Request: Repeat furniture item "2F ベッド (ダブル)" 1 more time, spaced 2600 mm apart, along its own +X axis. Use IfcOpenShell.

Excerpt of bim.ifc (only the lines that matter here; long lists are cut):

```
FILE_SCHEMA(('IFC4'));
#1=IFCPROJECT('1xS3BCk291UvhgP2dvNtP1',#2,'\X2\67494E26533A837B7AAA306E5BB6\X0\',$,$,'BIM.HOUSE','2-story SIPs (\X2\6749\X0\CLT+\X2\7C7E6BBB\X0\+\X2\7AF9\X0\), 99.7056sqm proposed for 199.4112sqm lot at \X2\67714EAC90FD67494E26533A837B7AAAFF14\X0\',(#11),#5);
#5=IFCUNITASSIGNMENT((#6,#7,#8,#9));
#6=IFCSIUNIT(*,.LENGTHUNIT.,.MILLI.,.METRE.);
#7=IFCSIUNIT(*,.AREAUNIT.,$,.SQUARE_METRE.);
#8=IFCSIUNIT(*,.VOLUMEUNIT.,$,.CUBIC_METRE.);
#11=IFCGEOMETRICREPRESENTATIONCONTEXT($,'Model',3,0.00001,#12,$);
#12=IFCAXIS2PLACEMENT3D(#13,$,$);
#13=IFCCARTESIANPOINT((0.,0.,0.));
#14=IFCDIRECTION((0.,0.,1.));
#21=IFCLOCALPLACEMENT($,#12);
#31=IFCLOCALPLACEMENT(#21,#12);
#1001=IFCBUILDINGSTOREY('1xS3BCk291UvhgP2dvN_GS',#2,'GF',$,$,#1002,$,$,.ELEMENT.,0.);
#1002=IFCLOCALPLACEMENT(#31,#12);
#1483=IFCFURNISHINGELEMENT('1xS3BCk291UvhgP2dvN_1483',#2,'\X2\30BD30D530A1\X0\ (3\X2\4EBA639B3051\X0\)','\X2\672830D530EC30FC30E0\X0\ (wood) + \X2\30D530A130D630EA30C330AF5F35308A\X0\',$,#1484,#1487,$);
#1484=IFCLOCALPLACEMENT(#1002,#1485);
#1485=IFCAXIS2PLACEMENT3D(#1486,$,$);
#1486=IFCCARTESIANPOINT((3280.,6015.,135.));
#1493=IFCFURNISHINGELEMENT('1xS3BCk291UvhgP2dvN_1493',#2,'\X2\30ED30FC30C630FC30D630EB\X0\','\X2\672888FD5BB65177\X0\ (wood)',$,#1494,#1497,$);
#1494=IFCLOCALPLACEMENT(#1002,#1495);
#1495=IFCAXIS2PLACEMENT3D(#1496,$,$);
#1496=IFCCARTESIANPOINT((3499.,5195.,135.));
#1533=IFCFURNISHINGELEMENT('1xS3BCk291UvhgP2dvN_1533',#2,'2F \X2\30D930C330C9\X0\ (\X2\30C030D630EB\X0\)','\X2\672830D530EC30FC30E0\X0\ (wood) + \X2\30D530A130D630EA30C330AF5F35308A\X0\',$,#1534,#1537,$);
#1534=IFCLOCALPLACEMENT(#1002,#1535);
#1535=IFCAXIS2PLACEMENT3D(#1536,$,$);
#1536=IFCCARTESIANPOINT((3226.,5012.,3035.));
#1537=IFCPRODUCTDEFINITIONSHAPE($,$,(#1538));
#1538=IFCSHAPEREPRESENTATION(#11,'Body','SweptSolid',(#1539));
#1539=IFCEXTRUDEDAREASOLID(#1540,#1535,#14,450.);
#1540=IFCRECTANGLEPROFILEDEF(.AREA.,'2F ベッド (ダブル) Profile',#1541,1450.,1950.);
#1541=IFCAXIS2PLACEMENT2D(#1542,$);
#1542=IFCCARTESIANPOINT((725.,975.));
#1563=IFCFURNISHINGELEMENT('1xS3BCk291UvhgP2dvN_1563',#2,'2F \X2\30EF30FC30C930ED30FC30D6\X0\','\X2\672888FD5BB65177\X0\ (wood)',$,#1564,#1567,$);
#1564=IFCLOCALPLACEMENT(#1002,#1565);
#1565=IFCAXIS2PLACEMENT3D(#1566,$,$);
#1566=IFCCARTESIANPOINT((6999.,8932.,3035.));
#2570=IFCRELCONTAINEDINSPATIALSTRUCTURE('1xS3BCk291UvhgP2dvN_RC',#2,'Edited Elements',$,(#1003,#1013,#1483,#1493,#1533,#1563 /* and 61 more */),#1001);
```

```python
import ifcopenshell
import ifcopenshell.api.geometry
import ifcopenshell.api.root
import ifcopenshell.util.element
import ifcopenshell.util.placement

model = ifcopenshell.open("bim.ifc")


def reuse_history(source, copy):
    """copy_class also copies each property set's owner history, people and application; keep the originals."""
    for rel in copy.IsDefinedBy:
        if rel.is_a("IfcRelDefinesByProperties") and (history := rel.RelatingPropertyDefinition.OwnerHistory):
            rel.RelatingPropertyDefinition.OwnerHistory = source.OwnerHistory
            ifcopenshell.util.element.remove_deep2(model, history)


source = model.by_guid("1xS3BCk291UvhgP2dvN_1533")
base = ifcopenshell.util.placement.get_local_placement(source.ObjectPlacement)
step = base[:3, 0] * 2600.0

for i in range(1, 2):
    copy = ifcopenshell.api.root.copy_class(model, product=source)
    copy.Representation = ifcopenshell.util.element.copy_deep(
        model, source.Representation, exclude=["IfcGeometricRepresentationContext", "IfcRepresentationMap"]
    )
    reuse_history(source, copy)
    matrix = base.copy()
    matrix[:3, 3] += i * step
    print("added at", matrix[:3, 3].round(3) + 0.0)
    ifcopenshell.api.geometry.edit_object_placement(model, product=copy, matrix=matrix, is_si=False)

model.write("bim_rev.ifc")
```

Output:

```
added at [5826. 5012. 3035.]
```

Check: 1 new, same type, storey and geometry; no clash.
